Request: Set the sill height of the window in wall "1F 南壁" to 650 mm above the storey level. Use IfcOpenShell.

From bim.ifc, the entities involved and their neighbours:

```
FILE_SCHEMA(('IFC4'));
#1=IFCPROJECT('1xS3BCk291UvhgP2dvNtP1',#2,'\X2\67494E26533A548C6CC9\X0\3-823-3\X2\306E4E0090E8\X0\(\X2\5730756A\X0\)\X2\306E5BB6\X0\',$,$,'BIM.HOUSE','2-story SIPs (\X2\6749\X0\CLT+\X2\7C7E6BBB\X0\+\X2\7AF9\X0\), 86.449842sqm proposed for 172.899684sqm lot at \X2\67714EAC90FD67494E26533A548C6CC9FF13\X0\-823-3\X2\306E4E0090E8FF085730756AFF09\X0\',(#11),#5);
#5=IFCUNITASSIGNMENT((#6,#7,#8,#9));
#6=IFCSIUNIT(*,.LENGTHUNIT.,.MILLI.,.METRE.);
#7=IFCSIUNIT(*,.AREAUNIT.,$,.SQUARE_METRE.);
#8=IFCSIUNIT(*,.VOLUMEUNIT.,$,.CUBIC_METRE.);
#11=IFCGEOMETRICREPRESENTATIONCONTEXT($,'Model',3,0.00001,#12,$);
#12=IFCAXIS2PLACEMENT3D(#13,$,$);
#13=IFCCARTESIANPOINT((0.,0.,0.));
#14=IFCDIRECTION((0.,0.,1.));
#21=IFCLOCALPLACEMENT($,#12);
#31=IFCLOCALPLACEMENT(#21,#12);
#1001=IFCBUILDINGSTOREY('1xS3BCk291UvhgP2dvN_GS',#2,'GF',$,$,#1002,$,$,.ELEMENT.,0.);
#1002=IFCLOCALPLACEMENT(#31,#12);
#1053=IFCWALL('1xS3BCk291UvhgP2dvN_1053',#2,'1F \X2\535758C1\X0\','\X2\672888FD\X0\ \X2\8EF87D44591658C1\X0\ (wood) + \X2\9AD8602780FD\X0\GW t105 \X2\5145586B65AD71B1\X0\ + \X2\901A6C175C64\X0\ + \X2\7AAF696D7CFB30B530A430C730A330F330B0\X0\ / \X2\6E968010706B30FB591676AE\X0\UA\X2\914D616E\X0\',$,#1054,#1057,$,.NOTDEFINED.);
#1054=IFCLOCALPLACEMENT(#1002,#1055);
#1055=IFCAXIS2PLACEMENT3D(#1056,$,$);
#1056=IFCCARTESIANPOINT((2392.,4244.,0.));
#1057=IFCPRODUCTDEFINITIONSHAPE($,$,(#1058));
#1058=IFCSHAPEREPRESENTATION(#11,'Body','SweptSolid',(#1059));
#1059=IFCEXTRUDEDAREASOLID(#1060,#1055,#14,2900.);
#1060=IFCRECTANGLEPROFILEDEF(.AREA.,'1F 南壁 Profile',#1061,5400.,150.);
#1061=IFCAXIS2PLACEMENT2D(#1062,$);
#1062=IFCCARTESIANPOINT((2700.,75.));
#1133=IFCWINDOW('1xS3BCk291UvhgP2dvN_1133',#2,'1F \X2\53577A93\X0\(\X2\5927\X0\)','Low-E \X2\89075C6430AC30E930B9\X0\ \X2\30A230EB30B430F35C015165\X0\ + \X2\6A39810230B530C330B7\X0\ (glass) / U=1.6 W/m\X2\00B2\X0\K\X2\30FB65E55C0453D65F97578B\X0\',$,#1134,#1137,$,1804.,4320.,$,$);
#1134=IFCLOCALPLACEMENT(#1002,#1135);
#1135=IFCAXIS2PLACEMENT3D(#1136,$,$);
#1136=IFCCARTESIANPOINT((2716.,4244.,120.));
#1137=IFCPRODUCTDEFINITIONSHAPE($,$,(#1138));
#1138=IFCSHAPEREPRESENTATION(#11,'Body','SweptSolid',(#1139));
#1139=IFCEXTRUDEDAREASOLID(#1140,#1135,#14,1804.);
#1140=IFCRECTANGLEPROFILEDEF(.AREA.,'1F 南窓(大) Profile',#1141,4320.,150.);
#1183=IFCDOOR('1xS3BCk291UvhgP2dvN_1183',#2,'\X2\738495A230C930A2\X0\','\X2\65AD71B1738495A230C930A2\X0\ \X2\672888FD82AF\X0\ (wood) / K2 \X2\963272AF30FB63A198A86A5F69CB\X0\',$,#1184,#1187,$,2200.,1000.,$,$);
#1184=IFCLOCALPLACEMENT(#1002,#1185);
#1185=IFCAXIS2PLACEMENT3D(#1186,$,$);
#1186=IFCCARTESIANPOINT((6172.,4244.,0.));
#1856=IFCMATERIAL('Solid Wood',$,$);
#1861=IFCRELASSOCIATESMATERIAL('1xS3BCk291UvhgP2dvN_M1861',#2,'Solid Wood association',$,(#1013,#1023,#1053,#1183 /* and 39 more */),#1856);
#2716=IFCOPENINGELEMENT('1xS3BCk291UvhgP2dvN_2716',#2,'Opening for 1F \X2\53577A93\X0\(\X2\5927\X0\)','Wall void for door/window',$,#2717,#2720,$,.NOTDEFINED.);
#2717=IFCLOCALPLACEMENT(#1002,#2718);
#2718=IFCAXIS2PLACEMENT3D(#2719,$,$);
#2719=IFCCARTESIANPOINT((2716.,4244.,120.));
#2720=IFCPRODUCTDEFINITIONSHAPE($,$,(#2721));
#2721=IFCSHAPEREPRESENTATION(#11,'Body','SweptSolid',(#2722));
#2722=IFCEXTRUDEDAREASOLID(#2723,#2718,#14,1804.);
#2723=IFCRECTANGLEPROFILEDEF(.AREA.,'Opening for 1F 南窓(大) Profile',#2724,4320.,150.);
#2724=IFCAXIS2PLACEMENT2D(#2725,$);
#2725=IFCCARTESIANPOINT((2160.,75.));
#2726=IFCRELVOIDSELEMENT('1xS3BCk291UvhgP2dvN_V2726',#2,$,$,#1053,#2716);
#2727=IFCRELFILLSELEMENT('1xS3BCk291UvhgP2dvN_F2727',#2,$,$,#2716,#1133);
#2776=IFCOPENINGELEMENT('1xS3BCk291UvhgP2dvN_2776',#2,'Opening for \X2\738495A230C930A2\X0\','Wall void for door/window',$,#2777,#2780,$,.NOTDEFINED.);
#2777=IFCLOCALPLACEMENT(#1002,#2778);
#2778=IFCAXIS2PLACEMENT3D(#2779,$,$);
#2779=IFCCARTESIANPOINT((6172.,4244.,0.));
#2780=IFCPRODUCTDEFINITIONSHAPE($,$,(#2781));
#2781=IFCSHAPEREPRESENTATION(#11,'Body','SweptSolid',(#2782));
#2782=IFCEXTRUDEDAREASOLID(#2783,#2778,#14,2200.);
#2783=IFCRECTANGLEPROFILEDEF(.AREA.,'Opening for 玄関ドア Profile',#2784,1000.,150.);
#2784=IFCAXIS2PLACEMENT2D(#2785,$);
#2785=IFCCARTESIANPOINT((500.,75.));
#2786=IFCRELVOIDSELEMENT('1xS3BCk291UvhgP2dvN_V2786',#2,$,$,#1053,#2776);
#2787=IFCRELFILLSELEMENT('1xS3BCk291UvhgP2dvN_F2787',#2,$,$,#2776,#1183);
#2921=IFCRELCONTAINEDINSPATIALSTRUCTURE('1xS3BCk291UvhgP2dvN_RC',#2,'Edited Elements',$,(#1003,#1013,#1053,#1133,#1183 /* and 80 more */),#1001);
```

```python
import numpy as np
import ifcopenshell
import ifcopenshell.api.geometry
import ifcopenshell.geom
import ifcopenshell.util.element
import ifcopenshell.util.placement
import ifcopenshell.util.shape
import ifcopenshell.util.unit

model = ifcopenshell.open("bim.ifc")
unit_scale = ifcopenshell.util.unit.calculate_unit_scale(model)

window = model.by_guid("1xS3BCk291UvhgP2dvN_1133")
opening = window.FillsVoids[0].RelatingOpeningElement
storey = ifcopenshell.util.element.get_container(window, ifc_class="IfcBuildingStorey")
level = ifcopenshell.util.placement.get_local_placement(storey.ObjectPlacement)[2, 3]

# The opening's origin need not be at the sill, so measure its lowest point.
shape = ifcopenshell.geom.create_shape(ifcopenshell.geom.settings(), opening)
bottom = ifcopenshell.util.shape.get_shape_bottom_elevation(shape, shape.geometry) / unit_scale
dz = level + 0.65 / unit_scale - bottom

shift = np.array([0.0, 0.0, dz])
# The window is not placed relative to its opening, so move both.
for product in (opening, window):
    matrix = ifcopenshell.util.placement.get_local_placement(product.ObjectPlacement)
    matrix[:3, 3] += shift
    ifcopenshell.api.geometry.edit_object_placement(model, product=product, matrix=matrix, is_si=False)

print(f"moved by {dz * unit_scale:+.3f} m")

model.write("bim_edited.ifc")
```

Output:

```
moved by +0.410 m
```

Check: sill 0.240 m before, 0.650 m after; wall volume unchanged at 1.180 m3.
